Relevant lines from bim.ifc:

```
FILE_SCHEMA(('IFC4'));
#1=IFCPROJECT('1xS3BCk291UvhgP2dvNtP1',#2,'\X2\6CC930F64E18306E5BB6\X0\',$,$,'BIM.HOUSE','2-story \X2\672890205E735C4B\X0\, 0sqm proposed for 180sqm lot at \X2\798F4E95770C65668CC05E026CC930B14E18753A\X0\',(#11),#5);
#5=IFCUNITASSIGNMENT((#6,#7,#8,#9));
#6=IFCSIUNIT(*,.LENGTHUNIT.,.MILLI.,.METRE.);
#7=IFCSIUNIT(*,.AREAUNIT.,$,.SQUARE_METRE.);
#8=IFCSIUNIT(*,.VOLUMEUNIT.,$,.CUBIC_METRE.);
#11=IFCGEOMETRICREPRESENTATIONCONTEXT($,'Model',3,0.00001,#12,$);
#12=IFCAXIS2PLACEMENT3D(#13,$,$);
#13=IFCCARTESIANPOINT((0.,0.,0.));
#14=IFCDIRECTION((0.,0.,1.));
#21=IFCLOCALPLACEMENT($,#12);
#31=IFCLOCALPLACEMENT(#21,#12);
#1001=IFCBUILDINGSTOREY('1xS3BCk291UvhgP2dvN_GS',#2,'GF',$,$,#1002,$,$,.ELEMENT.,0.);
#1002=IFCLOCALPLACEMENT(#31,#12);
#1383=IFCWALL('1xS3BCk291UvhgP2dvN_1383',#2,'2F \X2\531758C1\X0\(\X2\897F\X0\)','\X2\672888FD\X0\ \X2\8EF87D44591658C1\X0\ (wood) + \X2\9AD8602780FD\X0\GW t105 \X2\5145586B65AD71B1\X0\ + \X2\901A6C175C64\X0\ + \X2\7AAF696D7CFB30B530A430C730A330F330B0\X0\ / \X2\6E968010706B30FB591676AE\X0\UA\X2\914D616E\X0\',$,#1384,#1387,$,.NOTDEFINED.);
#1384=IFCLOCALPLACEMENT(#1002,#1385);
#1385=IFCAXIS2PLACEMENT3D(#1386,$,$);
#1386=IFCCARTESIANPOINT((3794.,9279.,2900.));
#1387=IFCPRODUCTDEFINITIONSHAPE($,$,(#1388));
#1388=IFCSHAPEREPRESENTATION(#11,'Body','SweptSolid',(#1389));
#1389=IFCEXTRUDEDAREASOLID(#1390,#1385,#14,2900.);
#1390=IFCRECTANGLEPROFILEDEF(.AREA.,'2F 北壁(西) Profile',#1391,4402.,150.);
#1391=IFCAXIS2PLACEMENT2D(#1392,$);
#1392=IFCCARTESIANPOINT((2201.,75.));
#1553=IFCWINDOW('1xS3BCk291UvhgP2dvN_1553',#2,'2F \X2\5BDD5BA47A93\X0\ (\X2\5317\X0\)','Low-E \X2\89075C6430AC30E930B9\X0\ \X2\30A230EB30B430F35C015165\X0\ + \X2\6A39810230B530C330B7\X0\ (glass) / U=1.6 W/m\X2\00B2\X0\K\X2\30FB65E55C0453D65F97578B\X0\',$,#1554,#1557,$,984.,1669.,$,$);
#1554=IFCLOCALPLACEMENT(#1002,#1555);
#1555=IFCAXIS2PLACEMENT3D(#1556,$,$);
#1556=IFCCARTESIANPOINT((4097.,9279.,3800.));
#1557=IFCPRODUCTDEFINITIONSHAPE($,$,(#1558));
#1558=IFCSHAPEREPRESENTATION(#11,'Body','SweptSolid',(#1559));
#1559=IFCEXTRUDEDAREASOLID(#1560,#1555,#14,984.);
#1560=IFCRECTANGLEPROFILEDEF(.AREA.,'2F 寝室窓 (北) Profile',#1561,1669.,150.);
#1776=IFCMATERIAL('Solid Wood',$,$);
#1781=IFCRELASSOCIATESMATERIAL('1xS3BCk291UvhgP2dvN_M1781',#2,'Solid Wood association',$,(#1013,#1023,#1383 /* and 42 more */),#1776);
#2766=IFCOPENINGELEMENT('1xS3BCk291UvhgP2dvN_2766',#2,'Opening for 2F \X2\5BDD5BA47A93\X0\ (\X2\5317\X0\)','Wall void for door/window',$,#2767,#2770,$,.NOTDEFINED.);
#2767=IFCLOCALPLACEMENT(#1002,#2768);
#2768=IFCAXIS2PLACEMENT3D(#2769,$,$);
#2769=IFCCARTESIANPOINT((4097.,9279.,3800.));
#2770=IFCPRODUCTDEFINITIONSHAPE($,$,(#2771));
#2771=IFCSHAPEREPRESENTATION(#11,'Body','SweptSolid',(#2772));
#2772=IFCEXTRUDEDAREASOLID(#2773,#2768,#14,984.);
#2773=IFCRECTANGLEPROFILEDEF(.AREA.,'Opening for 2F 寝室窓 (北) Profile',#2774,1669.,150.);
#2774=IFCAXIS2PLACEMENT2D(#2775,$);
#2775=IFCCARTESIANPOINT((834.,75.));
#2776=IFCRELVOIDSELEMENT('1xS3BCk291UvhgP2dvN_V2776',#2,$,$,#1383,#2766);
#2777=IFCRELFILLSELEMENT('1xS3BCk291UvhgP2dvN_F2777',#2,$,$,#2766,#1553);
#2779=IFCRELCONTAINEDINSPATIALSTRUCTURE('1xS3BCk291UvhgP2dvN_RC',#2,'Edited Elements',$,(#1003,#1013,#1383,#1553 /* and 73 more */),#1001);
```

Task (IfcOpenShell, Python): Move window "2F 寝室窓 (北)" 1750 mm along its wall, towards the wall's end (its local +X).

```python
import ifcopenshell
import ifcopenshell.api.geometry
import ifcopenshell.util.placement
import ifcopenshell.util.unit

model = ifcopenshell.open("bim.ifc")
unit_scale = ifcopenshell.util.unit.calculate_unit_scale(model)

window = model.by_id(1553)
opening = window.FillsVoids[0].RelatingOpeningElement
wall = opening.VoidsElements[0].RelatingBuildingElement

wall_matrix = ifcopenshell.util.placement.get_local_placement(wall.ObjectPlacement)
shift = wall_matrix[:3, 0] * 1.75 / unit_scale
before = ifcopenshell.util.placement.get_local_placement(window.ObjectPlacement)[:3, 3].copy()

# The window is not placed relative to its opening, so move both.
for product in (opening, window):
    matrix = ifcopenshell.util.placement.get_local_placement(product.ObjectPlacement)
    matrix[:3, 3] += shift
    ifcopenshell.api.geometry.edit_object_placement(model, product=product, matrix=matrix, is_si=False)

after = ifcopenshell.util.placement.get_local_placement(window.ObjectPlacement)[:3, 3]
print("window moved by", (after - before).round(3) + 0.0)

model.write("bim_edited.ifc")
```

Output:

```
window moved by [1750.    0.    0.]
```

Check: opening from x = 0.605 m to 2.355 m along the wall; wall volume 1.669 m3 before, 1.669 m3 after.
